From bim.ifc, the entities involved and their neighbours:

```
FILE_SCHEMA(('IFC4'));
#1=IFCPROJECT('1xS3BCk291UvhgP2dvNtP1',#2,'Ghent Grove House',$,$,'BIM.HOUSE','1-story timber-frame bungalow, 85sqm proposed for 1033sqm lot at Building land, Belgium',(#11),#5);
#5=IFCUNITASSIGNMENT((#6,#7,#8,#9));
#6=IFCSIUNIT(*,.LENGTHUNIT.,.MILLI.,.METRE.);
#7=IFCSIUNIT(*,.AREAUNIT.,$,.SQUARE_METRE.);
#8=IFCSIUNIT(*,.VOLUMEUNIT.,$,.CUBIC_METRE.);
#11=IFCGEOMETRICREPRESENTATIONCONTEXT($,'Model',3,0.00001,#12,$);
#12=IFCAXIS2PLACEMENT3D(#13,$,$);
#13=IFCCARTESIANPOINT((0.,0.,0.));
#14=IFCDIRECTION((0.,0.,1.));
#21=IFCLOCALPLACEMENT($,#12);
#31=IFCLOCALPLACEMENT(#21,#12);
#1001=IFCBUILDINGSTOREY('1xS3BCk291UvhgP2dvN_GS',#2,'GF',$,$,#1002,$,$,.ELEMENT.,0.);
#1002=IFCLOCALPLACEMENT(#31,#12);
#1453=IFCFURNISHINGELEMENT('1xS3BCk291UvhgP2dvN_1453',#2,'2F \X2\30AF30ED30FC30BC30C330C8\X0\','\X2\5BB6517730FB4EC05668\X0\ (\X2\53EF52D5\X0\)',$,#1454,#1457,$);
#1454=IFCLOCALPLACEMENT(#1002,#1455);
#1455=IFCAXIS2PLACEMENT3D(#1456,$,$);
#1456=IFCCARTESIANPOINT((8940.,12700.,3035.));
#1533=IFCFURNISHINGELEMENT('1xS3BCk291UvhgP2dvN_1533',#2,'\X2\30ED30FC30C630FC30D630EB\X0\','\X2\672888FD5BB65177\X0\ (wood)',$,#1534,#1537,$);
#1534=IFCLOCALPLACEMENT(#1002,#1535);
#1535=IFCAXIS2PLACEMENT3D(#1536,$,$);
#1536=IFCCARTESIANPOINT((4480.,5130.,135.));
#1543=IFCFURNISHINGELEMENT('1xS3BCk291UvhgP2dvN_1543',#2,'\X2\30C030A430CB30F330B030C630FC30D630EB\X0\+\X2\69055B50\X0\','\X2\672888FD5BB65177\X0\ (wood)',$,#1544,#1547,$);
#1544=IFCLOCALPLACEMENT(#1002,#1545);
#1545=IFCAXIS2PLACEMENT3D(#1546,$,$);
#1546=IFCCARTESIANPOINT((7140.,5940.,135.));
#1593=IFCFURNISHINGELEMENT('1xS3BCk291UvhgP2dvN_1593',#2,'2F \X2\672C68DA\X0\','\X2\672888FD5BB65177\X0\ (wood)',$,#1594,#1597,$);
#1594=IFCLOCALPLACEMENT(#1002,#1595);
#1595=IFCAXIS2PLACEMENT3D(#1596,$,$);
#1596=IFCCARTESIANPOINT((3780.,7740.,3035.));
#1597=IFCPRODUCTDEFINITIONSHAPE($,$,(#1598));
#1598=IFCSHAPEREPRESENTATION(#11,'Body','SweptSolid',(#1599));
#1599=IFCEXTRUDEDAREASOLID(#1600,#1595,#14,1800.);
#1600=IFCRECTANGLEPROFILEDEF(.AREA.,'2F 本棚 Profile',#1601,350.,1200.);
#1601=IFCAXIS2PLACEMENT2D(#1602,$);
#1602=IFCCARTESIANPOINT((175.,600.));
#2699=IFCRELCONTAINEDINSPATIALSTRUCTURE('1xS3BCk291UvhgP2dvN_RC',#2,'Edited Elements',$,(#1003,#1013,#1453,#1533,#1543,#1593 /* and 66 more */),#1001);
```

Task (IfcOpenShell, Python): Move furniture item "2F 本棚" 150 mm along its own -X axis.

```python
import ifcopenshell
import ifcopenshell.api.geometry
import ifcopenshell.util.placement

model = ifcopenshell.open("bim.ifc")

item = model.by_id(1593)
matrix = ifcopenshell.util.placement.get_local_placement(item.ObjectPlacement)
matrix[:3, 3] -= matrix[:3, 0] * 150.0
ifcopenshell.api.geometry.edit_object_placement(model, product=item, matrix=matrix, is_si=False)

print(ifcopenshell.util.placement.get_local_placement(item.ObjectPlacement).round(3) + 0.0)

model.write("bim_v2.ifc")
```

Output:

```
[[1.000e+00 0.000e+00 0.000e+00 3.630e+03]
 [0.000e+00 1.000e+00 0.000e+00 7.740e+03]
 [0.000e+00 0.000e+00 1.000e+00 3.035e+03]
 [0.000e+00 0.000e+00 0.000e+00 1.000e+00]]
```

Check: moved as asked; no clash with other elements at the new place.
